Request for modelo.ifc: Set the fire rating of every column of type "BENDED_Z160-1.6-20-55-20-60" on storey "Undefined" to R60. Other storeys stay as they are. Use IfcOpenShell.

First a look at what the model holds.

```python
import ifcopenshell
import ifcopenshell.util.element

model = ifcopenshell.open("modelo.ifc")
print(model.schema)
storey = next(s for s in model.by_type("IfcBuildingStorey") if s.Name == "Undefined")
columns = [e for e in ifcopenshell.util.element.get_decomposition(storey) if e.is_a("IfcColumn")]
seen = {}
for e in columns:
    element_type = ifcopenshell.util.element.get_type(e)
    key = (element_type.Name if element_type != e and element_type else None, ifcopenshell.util.element.get_pset(e, "Pset_ColumnCommon", "FireRating"))
    seen[key] = seen.get(key, 0) + 1
for (name, value), count in sorted(seen.items(), key=str):
    print(count, "x", name, "|", value)
```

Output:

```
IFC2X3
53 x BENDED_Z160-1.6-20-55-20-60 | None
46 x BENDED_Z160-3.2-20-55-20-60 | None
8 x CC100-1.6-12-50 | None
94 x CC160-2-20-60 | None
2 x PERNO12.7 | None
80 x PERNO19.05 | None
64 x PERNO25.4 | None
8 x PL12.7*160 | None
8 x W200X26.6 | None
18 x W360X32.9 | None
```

```python
import ifcopenshell
import ifcopenshell.api.pset
import ifcopenshell.util.element

model = ifcopenshell.open("modelo.ifc")

storey = next(s for s in model.by_type("IfcBuildingStorey") if s.Name == "Undefined")
columns = [e for e in ifcopenshell.util.element.get_decomposition(storey) if e.is_a("IfcColumn")]

count = 0
for e in columns:
    element_type = ifcopenshell.util.element.get_type(e)
    if element_type in (None, e) or element_type.Name != "BENDED_Z160-1.6-20-55-20-60":
        continue
    found = ifcopenshell.util.element.get_pset(e, "Pset_ColumnCommon", should_inherit=False)
    if found:
        pset = model.by_id(found["id"])
        if len(ifcopenshell.util.element.get_elements_by_pset(pset)) > 1:
            pset = ifcopenshell.api.pset.unshare_pset(model, products=[e], pset=pset)[0]
    else:
        pset = ifcopenshell.api.pset.add_pset(model, product=e, name="Pset_ColumnCommon")
    ifcopenshell.api.pset.edit_pset(model, pset=pset, properties={"FireRating": "R60"})
    count += 1

print(count, "columns updated")

model.write("modelo_v2.ifc")
```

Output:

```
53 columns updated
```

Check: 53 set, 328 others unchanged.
